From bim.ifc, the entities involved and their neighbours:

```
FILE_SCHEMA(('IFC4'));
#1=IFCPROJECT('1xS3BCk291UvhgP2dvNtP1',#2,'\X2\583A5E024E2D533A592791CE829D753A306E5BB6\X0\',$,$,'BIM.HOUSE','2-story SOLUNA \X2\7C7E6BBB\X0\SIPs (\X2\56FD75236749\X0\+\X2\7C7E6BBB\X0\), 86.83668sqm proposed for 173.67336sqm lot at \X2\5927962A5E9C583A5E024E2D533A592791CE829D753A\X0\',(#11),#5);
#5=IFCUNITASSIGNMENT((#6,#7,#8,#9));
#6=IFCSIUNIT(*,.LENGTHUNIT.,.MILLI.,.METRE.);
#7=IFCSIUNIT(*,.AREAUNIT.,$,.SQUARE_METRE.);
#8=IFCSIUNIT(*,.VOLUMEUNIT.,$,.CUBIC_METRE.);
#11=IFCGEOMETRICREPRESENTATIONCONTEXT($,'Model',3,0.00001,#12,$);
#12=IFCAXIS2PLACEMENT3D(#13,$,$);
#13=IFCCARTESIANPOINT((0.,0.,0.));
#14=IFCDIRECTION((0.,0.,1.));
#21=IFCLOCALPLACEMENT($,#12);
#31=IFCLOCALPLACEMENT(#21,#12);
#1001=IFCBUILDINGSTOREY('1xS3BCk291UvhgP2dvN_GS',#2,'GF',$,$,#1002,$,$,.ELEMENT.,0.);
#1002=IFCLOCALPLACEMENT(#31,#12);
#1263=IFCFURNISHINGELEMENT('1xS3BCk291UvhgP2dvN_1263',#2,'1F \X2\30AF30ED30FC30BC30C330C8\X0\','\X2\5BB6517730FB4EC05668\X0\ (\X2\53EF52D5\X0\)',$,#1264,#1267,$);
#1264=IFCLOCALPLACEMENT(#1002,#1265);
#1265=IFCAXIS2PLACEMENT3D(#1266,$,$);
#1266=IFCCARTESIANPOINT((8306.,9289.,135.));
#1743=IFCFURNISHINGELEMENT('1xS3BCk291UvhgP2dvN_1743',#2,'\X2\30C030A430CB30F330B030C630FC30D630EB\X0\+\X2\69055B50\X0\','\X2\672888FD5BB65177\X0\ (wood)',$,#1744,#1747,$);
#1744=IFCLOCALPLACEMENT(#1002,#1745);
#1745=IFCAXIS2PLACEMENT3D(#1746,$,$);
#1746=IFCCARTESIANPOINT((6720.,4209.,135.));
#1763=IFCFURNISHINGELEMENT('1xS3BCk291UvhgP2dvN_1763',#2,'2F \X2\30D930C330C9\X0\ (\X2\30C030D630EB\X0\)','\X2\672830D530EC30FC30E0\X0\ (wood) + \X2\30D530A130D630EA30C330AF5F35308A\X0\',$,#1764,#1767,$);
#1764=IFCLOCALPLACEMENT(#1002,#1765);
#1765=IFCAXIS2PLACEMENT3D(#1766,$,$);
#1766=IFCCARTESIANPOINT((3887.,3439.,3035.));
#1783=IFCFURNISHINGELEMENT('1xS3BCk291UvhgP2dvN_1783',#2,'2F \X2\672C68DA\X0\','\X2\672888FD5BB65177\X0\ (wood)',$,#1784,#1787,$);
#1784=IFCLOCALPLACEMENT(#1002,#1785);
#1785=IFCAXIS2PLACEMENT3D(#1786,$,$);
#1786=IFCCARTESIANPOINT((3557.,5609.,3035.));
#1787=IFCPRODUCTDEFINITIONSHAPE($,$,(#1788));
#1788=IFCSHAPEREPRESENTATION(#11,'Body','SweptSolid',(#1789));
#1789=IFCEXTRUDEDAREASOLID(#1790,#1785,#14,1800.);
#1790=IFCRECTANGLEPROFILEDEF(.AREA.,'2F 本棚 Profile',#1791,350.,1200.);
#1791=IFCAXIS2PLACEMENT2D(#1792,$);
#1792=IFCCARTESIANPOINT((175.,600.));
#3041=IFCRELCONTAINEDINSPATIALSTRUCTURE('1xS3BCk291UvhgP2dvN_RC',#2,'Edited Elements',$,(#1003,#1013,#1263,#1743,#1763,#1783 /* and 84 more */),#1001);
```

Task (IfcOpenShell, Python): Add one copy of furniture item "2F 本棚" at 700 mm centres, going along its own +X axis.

```python
import ifcopenshell
import ifcopenshell.api.geometry
import ifcopenshell.api.root
import ifcopenshell.util.element
import ifcopenshell.util.placement
import ifcopenshell.util.unit

model = ifcopenshell.open("bim.ifc")
unit_scale = ifcopenshell.util.unit.calculate_unit_scale(model)


def reuse_history(source, copy):
    """copy_class also copies each property set's owner history, people and application; keep the originals."""
    for rel in copy.IsDefinedBy:
        if rel.is_a("IfcRelDefinesByProperties") and (history := rel.RelatingPropertyDefinition.OwnerHistory):
            rel.RelatingPropertyDefinition.OwnerHistory = source.OwnerHistory
            ifcopenshell.util.element.remove_deep2(model, history)


source = model.by_guid("1xS3BCk291UvhgP2dvN_1783")
base = ifcopenshell.util.placement.get_local_placement(source.ObjectPlacement)
step = base[:3, 0] * 0.7 / unit_scale

for i in range(1, 2):
    copy = ifcopenshell.api.root.copy_class(model, product=source)
    copy.Representation = ifcopenshell.util.element.copy_deep(
        model, source.Representation, exclude=["IfcGeometricRepresentationContext", "IfcRepresentationMap"]
    )
    reuse_history(source, copy)
    matrix = base.copy()
    matrix[:3, 3] += i * step
    print("added at", matrix[:3, 3].round(3) + 0.0)
    ifcopenshell.api.geometry.edit_object_placement(model, product=copy, matrix=matrix, is_si=False)

model.write("bim_v2.ifc")
```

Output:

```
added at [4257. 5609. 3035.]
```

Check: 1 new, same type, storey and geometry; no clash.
